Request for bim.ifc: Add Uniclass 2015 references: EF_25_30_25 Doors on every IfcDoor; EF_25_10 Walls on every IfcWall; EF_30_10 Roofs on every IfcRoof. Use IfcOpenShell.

First a look at what the model holds.

```python
import ifcopenshell

model = ifcopenshell.open("bim.ifc")
print(model.schema)
print("classifications:", [c.Name for c in model.by_type("IfcClassification")])
for ifc_class in ("IfcDoor", "IfcRoof", "IfcStair", "IfcWall", "IfcWindow"):
    print(ifc_class, len(model.by_type(ifc_class)))
```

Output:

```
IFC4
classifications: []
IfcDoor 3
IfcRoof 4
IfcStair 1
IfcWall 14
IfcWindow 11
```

```python
import ifcopenshell
import ifcopenshell.api.classification

model = ifcopenshell.open("bim.ifc")

system = ifcopenshell.api.classification.add_classification(model, classification="Uniclass 2015")

codes = {
    "IfcDoor": ("EF_25_30_25", "Doors"),
    "IfcWall": ("EF_25_10", "Walls"),
    "IfcRoof": ("EF_30_10", "Roofs"),
}
for ifc_class, (code, name) in codes.items():
    products = model.by_type(ifc_class)
    ifcopenshell.api.classification.add_reference(
        model, products=products, classification=system, identification=code, name=name
    )
    print(code, len(products))

model.write("bim_rev.ifc")
```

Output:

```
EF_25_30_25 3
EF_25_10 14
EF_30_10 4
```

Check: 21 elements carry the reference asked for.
